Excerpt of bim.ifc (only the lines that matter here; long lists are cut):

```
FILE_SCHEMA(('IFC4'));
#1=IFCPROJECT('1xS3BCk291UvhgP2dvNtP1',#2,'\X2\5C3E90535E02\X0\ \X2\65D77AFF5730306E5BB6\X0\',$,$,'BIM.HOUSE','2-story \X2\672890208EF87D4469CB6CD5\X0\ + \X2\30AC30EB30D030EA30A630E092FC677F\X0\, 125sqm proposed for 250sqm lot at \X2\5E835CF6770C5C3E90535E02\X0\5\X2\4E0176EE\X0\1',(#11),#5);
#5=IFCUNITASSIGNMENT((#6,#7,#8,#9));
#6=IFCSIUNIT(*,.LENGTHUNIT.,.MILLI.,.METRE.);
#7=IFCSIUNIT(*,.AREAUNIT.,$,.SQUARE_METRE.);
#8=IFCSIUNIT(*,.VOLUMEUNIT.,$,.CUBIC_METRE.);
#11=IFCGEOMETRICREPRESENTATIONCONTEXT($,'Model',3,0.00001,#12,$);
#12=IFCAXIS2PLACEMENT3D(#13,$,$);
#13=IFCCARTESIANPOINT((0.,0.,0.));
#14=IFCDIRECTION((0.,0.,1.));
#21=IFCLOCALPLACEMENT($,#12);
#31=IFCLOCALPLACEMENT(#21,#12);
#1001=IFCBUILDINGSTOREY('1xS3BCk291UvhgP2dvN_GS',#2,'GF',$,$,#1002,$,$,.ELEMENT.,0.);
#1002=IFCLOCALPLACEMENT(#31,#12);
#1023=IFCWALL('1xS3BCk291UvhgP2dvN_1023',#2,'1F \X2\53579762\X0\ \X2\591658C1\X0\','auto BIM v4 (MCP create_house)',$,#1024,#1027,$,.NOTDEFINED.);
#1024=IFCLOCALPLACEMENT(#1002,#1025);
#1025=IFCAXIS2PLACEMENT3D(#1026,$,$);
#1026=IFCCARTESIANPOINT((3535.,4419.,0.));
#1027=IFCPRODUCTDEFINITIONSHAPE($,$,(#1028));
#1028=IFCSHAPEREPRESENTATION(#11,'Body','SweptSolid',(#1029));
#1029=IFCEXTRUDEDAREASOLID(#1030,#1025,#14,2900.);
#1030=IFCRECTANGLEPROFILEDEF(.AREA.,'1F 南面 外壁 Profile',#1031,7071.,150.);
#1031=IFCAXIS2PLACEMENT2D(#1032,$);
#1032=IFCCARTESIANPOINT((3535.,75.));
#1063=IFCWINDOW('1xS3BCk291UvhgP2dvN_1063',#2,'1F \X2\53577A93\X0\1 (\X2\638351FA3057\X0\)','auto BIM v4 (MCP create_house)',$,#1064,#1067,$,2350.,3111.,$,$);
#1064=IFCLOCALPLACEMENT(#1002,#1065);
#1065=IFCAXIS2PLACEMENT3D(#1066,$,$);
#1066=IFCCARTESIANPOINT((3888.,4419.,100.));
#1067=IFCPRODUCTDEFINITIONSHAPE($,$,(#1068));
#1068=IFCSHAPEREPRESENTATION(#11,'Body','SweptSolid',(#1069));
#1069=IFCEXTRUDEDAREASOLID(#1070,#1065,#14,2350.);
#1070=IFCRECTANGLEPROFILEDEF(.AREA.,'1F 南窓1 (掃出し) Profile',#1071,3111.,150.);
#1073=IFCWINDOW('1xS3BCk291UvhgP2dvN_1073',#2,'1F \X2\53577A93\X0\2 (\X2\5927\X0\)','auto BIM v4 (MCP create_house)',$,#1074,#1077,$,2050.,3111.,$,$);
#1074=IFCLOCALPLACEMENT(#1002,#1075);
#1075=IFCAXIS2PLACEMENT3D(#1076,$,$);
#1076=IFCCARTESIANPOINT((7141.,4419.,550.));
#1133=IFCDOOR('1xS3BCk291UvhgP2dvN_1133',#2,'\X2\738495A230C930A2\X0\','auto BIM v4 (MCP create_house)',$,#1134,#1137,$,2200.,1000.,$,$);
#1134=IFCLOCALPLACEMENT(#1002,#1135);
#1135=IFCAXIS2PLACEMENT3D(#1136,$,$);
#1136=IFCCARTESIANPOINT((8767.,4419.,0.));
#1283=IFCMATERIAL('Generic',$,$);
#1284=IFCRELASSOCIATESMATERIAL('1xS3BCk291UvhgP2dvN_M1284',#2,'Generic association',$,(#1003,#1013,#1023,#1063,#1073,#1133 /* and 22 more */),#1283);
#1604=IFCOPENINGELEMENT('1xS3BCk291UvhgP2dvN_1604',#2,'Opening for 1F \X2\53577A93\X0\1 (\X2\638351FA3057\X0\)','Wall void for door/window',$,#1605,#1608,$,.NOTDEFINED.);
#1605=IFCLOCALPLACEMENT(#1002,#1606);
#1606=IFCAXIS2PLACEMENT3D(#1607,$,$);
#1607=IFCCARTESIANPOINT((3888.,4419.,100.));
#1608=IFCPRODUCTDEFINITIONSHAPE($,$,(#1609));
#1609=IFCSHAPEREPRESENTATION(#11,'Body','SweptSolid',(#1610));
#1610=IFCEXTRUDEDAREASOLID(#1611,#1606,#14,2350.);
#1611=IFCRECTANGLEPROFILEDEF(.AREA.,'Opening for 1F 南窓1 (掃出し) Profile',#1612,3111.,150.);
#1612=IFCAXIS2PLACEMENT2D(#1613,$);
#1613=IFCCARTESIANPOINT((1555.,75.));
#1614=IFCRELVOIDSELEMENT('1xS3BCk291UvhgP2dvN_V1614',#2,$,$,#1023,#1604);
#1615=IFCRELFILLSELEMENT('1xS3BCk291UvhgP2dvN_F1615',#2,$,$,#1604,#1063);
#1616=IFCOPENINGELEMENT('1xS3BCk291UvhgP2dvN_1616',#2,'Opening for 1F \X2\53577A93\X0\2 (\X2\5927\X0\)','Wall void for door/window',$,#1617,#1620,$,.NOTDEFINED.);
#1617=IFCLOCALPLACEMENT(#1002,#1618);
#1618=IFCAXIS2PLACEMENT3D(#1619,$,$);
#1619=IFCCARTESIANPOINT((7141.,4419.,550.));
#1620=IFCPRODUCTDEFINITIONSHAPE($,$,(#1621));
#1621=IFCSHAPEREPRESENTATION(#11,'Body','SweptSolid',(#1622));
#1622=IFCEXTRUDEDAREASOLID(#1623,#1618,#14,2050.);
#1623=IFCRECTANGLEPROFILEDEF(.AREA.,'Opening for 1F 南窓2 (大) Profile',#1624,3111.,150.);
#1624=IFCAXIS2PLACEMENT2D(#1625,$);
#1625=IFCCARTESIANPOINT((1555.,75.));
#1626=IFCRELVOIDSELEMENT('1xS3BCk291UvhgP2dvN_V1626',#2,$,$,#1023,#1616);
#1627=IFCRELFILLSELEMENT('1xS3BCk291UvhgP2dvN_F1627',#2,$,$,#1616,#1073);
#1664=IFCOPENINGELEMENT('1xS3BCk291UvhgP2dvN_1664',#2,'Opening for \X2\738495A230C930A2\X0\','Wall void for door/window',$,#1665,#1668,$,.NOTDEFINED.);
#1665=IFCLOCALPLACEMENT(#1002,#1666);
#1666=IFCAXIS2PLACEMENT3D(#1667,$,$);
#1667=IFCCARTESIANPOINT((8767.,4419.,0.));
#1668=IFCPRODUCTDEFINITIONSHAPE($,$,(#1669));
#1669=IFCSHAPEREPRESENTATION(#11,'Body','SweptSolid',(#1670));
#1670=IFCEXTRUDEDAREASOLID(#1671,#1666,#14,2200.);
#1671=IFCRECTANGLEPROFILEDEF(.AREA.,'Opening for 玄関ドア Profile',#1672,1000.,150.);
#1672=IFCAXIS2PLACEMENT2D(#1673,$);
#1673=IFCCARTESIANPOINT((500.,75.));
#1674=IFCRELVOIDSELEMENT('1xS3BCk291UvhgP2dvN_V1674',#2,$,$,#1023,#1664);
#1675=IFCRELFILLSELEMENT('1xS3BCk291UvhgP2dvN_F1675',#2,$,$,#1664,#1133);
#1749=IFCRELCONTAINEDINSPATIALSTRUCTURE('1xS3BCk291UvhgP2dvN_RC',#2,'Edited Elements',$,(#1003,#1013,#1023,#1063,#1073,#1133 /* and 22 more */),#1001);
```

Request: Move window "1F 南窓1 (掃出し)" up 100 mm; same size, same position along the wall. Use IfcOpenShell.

```python
import numpy as np
import ifcopenshell
import ifcopenshell.api.geometry
import ifcopenshell.util.placement
import ifcopenshell.util.unit

model = ifcopenshell.open("bim.ifc")
unit_scale = ifcopenshell.util.unit.calculate_unit_scale(model)

window = model.by_guid("1xS3BCk291UvhgP2dvN_1063")
opening = window.FillsVoids[0].RelatingOpeningElement
dz = 100.0

shift = np.array([0.0, 0.0, dz])
# The window is not placed relative to its opening, so move both.
for product in (opening, window):
    matrix = ifcopenshell.util.placement.get_local_placement(product.ObjectPlacement)
    matrix[:3, 3] += shift
    ifcopenshell.api.geometry.edit_object_placement(model, product=product, matrix=matrix, is_si=False)

print(f"moved by {dz * unit_scale:+.3f} m")

model.write("bim_edited.ifc")
```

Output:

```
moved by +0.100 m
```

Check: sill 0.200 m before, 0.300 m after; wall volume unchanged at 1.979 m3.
